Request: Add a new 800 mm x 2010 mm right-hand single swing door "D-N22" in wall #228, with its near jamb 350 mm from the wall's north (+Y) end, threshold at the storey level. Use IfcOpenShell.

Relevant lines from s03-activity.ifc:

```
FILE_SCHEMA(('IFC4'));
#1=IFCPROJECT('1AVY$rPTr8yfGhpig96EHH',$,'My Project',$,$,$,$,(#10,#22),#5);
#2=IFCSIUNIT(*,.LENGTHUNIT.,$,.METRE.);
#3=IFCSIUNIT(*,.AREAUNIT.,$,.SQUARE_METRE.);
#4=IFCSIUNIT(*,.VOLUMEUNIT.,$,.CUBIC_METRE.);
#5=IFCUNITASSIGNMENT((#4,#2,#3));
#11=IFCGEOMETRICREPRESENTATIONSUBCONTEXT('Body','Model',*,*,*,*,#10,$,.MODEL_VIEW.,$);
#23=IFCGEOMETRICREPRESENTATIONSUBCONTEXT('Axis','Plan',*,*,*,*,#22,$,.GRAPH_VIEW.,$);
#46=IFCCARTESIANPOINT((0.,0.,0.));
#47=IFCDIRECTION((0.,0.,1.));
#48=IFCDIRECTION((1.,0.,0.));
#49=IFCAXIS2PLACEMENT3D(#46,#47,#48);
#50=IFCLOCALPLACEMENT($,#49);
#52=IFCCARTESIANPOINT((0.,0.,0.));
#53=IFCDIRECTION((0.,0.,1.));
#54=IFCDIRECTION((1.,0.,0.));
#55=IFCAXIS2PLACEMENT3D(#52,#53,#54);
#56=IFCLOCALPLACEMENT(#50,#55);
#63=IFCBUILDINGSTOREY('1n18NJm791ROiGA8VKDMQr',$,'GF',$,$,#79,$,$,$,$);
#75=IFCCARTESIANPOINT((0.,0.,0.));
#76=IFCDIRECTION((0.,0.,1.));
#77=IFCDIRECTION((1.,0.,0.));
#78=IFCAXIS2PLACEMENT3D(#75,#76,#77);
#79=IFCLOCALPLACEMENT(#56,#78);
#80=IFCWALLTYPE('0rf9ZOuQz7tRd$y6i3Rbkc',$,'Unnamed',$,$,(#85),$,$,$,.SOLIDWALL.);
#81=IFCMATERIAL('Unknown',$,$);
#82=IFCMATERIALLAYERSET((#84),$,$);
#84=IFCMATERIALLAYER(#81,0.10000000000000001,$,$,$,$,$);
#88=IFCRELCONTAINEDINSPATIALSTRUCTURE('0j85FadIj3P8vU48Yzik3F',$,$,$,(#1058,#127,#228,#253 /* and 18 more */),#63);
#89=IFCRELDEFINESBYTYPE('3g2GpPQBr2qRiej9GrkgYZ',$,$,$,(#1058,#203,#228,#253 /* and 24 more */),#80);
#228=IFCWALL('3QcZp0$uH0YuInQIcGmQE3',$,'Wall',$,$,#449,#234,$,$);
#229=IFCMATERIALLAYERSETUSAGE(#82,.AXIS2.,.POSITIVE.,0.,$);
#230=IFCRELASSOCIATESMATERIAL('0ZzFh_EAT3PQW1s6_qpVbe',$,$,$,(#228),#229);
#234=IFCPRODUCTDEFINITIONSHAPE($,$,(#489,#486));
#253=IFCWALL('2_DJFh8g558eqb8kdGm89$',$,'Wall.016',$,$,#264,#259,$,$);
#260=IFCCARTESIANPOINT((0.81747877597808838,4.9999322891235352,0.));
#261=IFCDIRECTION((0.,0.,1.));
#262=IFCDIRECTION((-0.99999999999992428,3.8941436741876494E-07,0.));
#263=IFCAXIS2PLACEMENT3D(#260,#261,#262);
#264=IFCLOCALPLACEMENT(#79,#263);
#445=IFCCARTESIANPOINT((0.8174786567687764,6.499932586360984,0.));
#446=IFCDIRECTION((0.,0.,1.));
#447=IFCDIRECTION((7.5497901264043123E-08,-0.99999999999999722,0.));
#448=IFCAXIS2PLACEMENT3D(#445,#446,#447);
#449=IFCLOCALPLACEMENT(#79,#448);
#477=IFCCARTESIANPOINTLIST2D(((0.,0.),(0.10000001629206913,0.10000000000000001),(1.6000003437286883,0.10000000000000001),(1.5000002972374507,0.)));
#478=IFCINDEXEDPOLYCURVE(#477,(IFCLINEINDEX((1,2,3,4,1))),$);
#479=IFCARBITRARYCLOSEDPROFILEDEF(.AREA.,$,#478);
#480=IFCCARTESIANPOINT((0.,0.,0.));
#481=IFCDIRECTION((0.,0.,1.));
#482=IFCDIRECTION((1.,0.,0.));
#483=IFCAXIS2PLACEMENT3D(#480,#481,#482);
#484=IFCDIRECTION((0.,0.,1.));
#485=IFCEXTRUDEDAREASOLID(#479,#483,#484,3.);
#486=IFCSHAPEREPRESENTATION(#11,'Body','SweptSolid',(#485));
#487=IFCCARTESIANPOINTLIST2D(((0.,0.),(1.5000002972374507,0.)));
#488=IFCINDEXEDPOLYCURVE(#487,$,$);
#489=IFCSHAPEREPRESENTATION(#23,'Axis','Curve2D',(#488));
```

```python
import numpy as np
import ifcopenshell
import ifcopenshell.api.feature
import ifcopenshell.api.geometry
import ifcopenshell.api.root
import ifcopenshell.api.spatial
import ifcopenshell.geom
import ifcopenshell.util.element
import ifcopenshell.util.placement
import ifcopenshell.util.representation
import ifcopenshell.util.shape
import ifcopenshell.util.unit

model = ifcopenshell.open("s03-activity.ifc")
unit_scale = ifcopenshell.util.unit.calculate_unit_scale(model)
settings = ifcopenshell.geom.settings()


def volume(element):
    """Net volume in cubic metres, openings subtracted."""
    shape = ifcopenshell.geom.create_shape(settings, element)
    return ifcopenshell.util.shape.get_volume(shape.geometry)


wall = model.by_guid("3QcZp0$uH0YuInQIcGmQE3")
storey = ifcopenshell.util.element.get_container(wall, ifc_class="IfcBuildingStorey")
context = ifcopenshell.util.representation.get_context(model, "Model", "Body", "MODEL_VIEW")
before = volume(wall)

width, height, from_end, sill = 0.8, 2.01, 0.35, 0.0  # metres

# The wall runs along its own X axis, and the end named is its -X end.
wall_shape = ifcopenshell.geom.create_shape(settings, wall)
x, y, z = ifcopenshell.util.shape.get_vertices(wall_shape.geometry).T
start = x.min() + from_end
face, thickness = float(y.min()), float(y.max() - y.min())
wall_matrix = ifcopenshell.util.placement.get_local_placement(wall.ObjectPlacement)
level = ifcopenshell.util.placement.get_local_placement(storey.ObjectPlacement)[2, 3]


def in_wall(x, y):
    """Placement at x, y metres in the wall's axes, at sill height."""
    matrix = wall_matrix.copy()
    matrix[:, 3] = wall_matrix @ np.array([x / unit_scale, y / unit_scale, 0.0, 1.0])
    matrix[2, 3] = level + sill / unit_scale
    return matrix


# Opening: a box that overshoots both wall faces by 50 mm.
opening = ifcopenshell.api.root.create_entity(model, ifc_class="IfcOpeningElement", predefined_type="OPENING")
box = ifcopenshell.api.geometry.add_wall_representation(
    model, context=context, length=width, height=height, thickness=thickness + 0.1
)
ifcopenshell.api.geometry.assign_representation(model, product=opening, representation=box)
ifcopenshell.api.geometry.edit_object_placement(model, product=opening, matrix=in_wall(start, face - 0.05), is_si=False)
ifcopenshell.api.feature.add_feature(model, feature=opening, element=wall)

door = ifcopenshell.api.root.create_entity(model, ifc_class="IfcDoor", name="D-N22", predefined_type="DOOR")
door.OverallWidth, door.OverallHeight = width / unit_scale, height / unit_scale
door.OperationType = "SINGLE_SWING_RIGHT"
body = ifcopenshell.api.geometry.add_door_representation(
    model,
    context=context,
    overall_width=door.OverallWidth,
    overall_height=door.OverallHeight,
    operation_type="SINGLE_SWING_RIGHT",
    lining_properties={"LiningDepth": thickness / unit_scale, "ThresholdDepth": thickness / unit_scale},
)
ifcopenshell.api.geometry.assign_representation(model, product=door, representation=body)
ifcopenshell.api.spatial.assign_container(model, products=[door], relating_structure=storey)
ifcopenshell.api.feature.add_filling(model, opening=opening, element=door)

# The lining spans the wall, so the door starts at the wall face.
ifcopenshell.api.geometry.edit_object_placement(model, product=door, matrix=in_wall(start, face), is_si=False)

after = volume(wall)

print(f"wall volume {before:.3f} -> {after:.3f} m3")

model.write("s03-activity_rev.ifc")
```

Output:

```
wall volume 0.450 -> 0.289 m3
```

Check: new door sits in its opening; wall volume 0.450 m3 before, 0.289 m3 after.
